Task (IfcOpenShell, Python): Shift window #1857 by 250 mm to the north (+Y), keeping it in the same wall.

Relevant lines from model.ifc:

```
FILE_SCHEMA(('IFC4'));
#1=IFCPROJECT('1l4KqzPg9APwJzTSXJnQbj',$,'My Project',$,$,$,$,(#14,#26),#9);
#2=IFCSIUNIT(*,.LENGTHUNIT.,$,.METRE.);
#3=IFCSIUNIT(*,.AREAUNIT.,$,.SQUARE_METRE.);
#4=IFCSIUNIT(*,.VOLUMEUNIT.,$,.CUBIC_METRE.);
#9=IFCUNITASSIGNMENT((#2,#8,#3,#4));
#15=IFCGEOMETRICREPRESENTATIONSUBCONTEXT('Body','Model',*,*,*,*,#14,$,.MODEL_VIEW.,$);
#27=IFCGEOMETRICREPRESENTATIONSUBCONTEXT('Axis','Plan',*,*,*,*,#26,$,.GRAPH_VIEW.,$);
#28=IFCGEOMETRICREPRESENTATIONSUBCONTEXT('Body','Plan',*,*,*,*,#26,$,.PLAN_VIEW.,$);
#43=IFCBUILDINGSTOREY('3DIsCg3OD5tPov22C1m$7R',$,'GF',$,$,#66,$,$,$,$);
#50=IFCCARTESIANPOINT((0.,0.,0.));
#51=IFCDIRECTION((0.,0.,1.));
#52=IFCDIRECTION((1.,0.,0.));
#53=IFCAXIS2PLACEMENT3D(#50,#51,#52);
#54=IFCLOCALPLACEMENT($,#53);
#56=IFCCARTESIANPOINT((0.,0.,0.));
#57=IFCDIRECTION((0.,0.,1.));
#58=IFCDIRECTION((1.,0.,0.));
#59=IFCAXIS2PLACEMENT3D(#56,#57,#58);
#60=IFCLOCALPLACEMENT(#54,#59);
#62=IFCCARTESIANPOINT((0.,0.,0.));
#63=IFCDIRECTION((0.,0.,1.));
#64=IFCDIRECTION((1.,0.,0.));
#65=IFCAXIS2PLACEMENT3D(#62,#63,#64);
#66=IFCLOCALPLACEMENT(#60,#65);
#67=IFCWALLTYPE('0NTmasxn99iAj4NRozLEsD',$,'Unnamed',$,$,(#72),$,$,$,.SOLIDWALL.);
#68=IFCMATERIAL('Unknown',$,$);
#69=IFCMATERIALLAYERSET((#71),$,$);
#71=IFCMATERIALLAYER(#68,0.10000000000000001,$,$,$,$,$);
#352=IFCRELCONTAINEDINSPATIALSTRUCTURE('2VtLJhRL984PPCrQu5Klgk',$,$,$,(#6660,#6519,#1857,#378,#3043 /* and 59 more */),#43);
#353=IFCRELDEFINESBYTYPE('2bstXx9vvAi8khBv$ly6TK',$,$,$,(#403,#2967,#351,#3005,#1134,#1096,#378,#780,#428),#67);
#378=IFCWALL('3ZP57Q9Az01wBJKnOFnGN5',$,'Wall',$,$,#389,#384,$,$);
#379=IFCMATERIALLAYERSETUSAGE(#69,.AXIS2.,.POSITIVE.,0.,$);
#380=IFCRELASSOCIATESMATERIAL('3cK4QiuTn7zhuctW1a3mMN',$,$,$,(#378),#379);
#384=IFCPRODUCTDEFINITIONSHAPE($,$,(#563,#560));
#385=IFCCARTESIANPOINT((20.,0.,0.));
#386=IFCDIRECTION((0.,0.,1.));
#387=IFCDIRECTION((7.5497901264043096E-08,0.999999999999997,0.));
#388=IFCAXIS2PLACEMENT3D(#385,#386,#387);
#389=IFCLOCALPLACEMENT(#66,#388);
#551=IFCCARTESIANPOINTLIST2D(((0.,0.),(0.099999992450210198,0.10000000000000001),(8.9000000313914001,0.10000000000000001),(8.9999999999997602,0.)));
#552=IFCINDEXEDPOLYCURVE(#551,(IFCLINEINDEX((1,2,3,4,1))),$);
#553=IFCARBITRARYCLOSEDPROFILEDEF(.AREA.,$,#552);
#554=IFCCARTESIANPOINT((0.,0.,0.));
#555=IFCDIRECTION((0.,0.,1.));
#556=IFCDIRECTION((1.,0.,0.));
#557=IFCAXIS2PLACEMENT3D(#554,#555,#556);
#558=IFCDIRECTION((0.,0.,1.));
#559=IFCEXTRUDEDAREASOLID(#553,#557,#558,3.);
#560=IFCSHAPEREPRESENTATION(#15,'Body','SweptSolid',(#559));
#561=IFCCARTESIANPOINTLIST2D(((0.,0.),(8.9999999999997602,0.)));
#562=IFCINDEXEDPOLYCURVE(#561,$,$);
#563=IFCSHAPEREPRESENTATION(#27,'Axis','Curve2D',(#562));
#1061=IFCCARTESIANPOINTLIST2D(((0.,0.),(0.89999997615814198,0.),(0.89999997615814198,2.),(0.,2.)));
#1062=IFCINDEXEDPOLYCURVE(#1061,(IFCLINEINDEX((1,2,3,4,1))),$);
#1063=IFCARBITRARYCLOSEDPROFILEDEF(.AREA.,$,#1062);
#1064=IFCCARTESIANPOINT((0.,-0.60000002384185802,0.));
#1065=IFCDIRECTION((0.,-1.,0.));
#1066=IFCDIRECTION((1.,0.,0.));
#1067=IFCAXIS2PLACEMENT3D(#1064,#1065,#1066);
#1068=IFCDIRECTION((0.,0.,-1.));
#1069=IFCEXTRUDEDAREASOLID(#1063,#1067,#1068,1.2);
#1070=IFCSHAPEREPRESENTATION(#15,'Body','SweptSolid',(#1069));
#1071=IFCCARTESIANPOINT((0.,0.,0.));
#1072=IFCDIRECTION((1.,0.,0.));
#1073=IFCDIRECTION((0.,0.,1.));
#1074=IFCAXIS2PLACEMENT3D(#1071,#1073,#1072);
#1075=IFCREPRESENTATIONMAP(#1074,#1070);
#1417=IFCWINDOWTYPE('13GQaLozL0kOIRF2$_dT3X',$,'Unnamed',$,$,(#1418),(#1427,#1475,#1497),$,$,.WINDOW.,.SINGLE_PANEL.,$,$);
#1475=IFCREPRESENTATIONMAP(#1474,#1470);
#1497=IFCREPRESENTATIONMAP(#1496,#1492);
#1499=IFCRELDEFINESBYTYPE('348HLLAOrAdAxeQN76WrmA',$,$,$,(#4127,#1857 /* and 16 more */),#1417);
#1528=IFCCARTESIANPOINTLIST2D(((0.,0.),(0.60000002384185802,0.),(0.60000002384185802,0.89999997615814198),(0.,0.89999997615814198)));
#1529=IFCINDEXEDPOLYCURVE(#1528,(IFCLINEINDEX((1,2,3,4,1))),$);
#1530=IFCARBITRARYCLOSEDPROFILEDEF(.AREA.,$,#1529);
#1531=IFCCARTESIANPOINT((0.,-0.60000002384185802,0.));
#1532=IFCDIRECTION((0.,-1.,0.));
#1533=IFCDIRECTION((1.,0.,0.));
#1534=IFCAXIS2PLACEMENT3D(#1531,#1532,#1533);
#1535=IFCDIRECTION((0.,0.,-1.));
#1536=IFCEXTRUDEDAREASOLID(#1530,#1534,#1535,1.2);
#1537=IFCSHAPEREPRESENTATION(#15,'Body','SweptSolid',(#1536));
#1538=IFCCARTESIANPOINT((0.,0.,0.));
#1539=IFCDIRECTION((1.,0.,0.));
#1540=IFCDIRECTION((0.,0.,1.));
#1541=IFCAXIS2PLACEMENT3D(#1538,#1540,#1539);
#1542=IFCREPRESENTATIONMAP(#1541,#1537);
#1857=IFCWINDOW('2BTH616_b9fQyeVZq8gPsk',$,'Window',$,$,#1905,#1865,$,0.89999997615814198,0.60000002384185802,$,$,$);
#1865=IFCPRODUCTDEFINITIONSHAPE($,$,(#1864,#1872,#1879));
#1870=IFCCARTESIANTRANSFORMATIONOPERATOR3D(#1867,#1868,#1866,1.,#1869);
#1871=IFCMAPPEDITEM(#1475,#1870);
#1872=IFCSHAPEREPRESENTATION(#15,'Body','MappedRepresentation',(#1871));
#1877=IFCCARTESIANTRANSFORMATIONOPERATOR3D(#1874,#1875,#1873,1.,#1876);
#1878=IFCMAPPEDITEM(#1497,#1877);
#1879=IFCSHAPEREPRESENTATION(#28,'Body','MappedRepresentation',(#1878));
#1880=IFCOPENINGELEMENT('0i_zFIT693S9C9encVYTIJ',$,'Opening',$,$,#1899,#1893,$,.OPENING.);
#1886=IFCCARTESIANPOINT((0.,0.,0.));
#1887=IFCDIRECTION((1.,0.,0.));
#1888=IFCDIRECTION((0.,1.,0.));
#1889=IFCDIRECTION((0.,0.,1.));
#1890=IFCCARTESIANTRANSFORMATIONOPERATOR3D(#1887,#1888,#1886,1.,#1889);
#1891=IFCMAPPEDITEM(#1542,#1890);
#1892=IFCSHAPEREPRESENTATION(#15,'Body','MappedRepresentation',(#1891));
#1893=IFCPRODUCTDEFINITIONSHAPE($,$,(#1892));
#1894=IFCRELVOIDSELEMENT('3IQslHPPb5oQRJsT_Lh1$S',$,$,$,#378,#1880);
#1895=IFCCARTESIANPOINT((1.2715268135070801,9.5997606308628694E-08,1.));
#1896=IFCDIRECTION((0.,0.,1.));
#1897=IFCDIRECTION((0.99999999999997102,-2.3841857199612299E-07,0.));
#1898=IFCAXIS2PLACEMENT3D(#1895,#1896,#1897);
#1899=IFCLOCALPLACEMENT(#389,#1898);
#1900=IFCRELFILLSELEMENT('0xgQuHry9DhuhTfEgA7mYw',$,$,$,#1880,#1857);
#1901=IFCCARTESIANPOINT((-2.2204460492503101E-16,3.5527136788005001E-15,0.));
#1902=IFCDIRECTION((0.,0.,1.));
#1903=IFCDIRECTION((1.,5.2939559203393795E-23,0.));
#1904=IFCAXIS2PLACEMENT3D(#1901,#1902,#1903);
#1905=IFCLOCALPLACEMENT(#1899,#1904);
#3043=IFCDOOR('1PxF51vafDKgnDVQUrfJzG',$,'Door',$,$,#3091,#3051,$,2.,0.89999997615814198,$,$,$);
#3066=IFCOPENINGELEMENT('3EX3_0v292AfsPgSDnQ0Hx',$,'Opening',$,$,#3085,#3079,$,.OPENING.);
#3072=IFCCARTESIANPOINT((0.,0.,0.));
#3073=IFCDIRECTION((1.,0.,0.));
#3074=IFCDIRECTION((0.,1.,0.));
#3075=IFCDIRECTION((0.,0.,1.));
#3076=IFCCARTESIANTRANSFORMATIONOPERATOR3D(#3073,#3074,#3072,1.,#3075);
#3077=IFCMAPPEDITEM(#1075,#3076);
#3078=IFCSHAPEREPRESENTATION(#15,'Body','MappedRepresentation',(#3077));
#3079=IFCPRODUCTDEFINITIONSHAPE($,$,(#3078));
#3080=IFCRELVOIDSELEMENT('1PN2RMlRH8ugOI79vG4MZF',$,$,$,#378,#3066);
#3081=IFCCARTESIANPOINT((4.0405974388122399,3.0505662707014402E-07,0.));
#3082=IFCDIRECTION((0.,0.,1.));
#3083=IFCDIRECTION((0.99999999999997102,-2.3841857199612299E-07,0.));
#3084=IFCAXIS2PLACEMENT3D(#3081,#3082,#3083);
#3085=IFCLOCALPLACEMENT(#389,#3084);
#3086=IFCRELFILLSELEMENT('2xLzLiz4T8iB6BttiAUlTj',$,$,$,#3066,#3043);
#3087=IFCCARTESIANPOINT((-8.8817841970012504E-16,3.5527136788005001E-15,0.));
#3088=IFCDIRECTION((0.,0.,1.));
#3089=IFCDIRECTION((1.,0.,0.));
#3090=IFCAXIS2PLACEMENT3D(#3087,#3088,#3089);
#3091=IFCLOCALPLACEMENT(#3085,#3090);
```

```python
import ifcopenshell
import ifcopenshell.api.geometry
import ifcopenshell.util.placement

model = ifcopenshell.open("model.ifc")

window = model.by_guid("2BTH616_b9fQyeVZq8gPsk")
opening = window.FillsVoids[0].RelatingOpeningElement
wall = opening.VoidsElements[0].RelatingBuildingElement

wall_matrix = ifcopenshell.util.placement.get_local_placement(wall.ObjectPlacement)
shift = wall_matrix[:3, 0] * 0.25
before = ifcopenshell.util.placement.get_local_placement(window.ObjectPlacement)[:3, 3].copy()

# The window is placed relative to its opening, so it follows when the opening moves.
matrix = ifcopenshell.util.placement.get_local_placement(opening.ObjectPlacement)
matrix[:3, 3] += shift
ifcopenshell.api.geometry.edit_object_placement(
    model, product=opening, matrix=matrix, is_si=False, should_transform_children=True
)

after = ifcopenshell.util.placement.get_local_placement(window.ObjectPlacement)[:3, 3]
print("window moved by", (after - before).round(3) + 0.0)

model.write("model-out.ifc")
```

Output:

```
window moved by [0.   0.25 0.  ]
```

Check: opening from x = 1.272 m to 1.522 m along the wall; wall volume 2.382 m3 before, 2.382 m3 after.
